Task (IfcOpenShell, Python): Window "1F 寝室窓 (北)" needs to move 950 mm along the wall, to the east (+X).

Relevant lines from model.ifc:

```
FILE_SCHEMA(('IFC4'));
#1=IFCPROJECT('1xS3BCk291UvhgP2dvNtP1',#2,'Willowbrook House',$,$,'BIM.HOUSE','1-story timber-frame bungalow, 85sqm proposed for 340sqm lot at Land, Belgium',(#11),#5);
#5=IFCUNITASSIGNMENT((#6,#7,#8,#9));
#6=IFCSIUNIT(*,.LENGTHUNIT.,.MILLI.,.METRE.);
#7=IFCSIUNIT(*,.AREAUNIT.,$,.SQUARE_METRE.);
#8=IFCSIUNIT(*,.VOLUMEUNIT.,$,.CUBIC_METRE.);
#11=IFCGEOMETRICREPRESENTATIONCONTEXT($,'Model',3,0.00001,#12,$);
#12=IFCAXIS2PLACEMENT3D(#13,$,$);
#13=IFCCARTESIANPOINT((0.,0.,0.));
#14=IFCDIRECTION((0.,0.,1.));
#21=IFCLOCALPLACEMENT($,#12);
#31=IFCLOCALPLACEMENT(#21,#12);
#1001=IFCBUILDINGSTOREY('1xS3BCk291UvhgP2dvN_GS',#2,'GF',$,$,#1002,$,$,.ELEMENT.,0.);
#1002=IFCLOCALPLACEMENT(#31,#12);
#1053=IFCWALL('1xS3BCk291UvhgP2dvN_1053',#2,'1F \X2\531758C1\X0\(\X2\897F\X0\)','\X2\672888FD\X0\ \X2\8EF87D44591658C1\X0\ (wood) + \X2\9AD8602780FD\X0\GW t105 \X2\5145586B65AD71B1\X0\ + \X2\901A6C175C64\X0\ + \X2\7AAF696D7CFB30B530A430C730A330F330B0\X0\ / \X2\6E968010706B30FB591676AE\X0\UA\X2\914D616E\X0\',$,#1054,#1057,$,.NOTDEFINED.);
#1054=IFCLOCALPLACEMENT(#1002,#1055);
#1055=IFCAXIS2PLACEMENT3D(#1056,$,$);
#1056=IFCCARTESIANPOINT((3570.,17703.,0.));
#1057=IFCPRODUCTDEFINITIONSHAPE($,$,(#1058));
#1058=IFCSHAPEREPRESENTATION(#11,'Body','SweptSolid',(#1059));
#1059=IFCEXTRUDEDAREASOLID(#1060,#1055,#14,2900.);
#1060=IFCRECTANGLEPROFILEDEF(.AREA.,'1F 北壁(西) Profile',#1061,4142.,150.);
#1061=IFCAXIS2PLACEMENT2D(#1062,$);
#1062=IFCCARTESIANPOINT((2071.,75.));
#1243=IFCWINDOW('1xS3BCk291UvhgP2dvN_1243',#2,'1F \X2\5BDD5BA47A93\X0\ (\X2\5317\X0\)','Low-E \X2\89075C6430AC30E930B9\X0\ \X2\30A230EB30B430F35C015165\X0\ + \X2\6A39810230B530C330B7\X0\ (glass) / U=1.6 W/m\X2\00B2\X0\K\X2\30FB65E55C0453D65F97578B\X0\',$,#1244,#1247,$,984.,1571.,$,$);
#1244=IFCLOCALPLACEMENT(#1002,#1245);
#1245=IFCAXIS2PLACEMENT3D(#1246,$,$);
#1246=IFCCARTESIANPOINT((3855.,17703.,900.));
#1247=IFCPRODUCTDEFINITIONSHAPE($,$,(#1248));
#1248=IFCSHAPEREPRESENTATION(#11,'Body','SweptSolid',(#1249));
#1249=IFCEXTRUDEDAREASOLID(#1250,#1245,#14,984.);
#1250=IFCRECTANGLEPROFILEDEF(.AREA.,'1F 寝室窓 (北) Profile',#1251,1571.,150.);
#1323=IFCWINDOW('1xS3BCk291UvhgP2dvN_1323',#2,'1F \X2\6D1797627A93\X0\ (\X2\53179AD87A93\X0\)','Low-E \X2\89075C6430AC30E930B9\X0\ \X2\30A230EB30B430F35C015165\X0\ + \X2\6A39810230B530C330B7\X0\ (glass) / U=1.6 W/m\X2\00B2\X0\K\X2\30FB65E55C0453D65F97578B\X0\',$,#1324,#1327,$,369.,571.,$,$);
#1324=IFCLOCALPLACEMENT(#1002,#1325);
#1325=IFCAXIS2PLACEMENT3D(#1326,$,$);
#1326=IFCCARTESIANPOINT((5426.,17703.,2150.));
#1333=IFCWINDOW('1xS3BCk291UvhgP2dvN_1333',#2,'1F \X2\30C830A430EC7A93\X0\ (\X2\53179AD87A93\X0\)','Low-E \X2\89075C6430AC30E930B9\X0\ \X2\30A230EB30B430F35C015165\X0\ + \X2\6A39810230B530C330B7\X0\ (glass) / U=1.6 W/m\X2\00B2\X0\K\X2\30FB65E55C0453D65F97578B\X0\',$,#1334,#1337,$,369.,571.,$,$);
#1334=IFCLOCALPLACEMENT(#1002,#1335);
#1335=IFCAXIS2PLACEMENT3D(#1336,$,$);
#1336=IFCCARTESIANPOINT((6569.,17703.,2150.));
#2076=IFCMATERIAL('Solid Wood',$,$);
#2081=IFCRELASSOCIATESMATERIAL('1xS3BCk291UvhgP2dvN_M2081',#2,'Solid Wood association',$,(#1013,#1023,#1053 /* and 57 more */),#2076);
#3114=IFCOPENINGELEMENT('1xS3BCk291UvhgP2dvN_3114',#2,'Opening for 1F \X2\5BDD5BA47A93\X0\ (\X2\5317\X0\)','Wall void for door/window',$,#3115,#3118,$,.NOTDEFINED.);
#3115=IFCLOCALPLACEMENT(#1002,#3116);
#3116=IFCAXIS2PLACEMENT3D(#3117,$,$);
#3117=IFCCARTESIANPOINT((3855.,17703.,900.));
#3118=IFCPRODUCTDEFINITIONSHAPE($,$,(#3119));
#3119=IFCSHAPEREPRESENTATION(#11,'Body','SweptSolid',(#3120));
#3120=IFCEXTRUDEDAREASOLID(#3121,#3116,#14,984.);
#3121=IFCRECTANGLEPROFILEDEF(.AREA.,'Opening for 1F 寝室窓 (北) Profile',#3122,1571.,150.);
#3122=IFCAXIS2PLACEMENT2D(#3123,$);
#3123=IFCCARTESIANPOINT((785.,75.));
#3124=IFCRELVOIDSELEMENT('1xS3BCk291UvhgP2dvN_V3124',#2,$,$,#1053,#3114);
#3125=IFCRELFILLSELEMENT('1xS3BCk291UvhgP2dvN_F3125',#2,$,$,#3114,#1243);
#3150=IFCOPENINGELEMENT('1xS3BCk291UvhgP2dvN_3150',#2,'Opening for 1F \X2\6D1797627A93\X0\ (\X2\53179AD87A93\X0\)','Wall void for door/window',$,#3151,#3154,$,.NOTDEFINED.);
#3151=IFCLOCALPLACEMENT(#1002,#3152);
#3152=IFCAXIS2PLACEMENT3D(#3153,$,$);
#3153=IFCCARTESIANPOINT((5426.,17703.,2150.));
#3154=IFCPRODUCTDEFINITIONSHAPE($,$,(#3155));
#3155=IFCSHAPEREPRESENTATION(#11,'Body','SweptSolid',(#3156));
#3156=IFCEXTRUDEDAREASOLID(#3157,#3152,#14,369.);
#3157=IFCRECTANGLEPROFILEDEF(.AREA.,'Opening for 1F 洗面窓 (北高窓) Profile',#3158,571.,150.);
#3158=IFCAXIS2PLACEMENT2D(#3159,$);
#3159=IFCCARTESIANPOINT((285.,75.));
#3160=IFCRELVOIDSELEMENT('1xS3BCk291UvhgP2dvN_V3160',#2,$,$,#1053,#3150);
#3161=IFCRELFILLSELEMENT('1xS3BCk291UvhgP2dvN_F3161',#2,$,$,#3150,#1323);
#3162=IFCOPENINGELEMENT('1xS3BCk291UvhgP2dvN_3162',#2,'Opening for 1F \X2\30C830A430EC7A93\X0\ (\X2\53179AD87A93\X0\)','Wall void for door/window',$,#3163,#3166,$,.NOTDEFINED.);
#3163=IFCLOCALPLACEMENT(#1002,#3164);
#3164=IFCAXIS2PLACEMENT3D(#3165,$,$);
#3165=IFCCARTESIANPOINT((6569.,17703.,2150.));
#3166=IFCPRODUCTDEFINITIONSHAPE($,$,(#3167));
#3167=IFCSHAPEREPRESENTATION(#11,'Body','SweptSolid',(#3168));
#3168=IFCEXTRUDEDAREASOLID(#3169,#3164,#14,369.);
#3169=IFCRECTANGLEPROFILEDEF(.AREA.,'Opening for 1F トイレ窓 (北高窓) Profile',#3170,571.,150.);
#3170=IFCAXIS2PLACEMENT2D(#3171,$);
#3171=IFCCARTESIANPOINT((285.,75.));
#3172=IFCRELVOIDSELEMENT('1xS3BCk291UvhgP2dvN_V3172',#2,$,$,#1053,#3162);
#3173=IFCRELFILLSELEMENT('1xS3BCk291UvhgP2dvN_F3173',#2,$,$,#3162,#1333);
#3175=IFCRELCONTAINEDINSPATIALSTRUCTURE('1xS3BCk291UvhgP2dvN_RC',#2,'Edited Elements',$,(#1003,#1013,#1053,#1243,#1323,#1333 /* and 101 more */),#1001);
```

```python
import ifcopenshell
import ifcopenshell.api.geometry
import ifcopenshell.util.placement

model = ifcopenshell.open("model.ifc")

window = model.by_guid("1xS3BCk291UvhgP2dvN_1243")
opening = window.FillsVoids[0].RelatingOpeningElement
wall = opening.VoidsElements[0].RelatingBuildingElement

wall_matrix = ifcopenshell.util.placement.get_local_placement(wall.ObjectPlacement)
shift = wall_matrix[:3, 0] * 950.0
before = ifcopenshell.util.placement.get_local_placement(window.ObjectPlacement)[:3, 3].copy()

# The window is not placed relative to its opening, so move both.
for product in (opening, window):
    matrix = ifcopenshell.util.placement.get_local_placement(product.ObjectPlacement)
    matrix[:3, 3] += shift
    ifcopenshell.api.geometry.edit_object_placement(model, product=product, matrix=matrix, is_si=False)

after = ifcopenshell.util.placement.get_local_placement(window.ObjectPlacement)[:3, 3]
print("window moved by", (after - before).round(3) + 0.0)

model.write("model-out.ifc")
```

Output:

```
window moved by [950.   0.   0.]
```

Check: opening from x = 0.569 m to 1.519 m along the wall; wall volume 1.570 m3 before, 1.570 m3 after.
